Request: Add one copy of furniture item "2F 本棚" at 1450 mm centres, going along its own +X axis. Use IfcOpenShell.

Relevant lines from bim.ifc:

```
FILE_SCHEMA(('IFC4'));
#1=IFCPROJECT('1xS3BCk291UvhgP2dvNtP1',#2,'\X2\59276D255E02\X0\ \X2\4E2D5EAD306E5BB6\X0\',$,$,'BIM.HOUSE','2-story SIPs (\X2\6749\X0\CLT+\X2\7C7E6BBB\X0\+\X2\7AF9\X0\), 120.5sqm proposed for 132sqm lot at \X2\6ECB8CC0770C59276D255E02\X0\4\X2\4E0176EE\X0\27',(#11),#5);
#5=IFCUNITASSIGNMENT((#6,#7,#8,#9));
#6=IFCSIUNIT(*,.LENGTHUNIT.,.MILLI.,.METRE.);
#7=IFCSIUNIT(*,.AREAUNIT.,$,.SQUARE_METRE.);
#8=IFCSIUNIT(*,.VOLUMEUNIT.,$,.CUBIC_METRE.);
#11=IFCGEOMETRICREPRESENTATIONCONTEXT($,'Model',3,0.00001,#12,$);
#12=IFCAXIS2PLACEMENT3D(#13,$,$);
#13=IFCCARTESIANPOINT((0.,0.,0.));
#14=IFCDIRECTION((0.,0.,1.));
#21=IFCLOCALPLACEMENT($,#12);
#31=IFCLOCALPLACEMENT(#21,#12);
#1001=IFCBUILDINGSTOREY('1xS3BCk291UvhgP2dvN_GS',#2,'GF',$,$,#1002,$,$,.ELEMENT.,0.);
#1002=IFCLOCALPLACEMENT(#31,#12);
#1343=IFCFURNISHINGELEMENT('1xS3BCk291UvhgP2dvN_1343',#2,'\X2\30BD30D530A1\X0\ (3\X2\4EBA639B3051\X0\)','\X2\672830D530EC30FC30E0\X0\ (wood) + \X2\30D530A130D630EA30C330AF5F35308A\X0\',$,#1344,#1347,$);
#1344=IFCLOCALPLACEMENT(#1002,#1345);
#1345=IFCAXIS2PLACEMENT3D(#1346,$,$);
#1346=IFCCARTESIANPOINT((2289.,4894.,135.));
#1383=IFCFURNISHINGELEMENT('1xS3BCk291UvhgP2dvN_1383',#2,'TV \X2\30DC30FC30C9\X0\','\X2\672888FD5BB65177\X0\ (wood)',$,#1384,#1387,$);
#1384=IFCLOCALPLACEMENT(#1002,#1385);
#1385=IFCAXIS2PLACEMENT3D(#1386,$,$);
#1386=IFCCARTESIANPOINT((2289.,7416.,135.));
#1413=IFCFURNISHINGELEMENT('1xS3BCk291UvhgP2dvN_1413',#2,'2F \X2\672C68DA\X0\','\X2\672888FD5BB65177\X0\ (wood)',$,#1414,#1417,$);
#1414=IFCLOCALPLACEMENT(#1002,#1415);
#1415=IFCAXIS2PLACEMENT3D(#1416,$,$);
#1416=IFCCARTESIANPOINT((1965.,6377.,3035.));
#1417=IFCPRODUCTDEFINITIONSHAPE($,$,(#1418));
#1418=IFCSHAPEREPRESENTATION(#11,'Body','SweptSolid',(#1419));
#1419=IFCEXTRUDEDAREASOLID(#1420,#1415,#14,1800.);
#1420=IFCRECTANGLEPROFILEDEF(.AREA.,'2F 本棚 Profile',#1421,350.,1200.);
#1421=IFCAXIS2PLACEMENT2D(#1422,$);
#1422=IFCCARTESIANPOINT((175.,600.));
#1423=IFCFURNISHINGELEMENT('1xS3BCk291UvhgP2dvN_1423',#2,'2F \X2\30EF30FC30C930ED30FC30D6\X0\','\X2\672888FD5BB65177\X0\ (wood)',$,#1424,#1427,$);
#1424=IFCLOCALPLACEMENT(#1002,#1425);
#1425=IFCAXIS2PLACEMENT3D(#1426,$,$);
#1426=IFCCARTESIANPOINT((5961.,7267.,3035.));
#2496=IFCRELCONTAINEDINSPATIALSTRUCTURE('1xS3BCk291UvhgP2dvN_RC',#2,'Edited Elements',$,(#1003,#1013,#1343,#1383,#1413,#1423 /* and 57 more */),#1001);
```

```python
import ifcopenshell
import ifcopenshell.api.geometry
import ifcopenshell.api.root
import ifcopenshell.util.element
import ifcopenshell.util.placement

model = ifcopenshell.open("bim.ifc")


def reuse_history(source, copy):
    """copy_class also copies each property set's owner history, people and application; keep the originals."""
    for rel in copy.IsDefinedBy:
        if rel.is_a("IfcRelDefinesByProperties") and (history := rel.RelatingPropertyDefinition.OwnerHistory):
            rel.RelatingPropertyDefinition.OwnerHistory = source.OwnerHistory
            ifcopenshell.util.element.remove_deep2(model, history)


source = model.by_guid("1xS3BCk291UvhgP2dvN_1413")
base = ifcopenshell.util.placement.get_local_placement(source.ObjectPlacement)
step = base[:3, 0] * 1450.0

for i in range(1, 2):
    copy = ifcopenshell.api.root.copy_class(model, product=source)
    copy.Representation = ifcopenshell.util.element.copy_deep(
        model, source.Representation, exclude=["IfcGeometricRepresentationContext", "IfcRepresentationMap"]
    )
    reuse_history(source, copy)
    matrix = base.copy()
    matrix[:3, 3] += i * step
    print("added at", matrix[:3, 3].round(3) + 0.0)
    ifcopenshell.api.geometry.edit_object_placement(model, product=copy, matrix=matrix, is_si=False)

model.write("bim_updated.ifc")
```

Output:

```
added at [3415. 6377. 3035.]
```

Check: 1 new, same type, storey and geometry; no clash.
